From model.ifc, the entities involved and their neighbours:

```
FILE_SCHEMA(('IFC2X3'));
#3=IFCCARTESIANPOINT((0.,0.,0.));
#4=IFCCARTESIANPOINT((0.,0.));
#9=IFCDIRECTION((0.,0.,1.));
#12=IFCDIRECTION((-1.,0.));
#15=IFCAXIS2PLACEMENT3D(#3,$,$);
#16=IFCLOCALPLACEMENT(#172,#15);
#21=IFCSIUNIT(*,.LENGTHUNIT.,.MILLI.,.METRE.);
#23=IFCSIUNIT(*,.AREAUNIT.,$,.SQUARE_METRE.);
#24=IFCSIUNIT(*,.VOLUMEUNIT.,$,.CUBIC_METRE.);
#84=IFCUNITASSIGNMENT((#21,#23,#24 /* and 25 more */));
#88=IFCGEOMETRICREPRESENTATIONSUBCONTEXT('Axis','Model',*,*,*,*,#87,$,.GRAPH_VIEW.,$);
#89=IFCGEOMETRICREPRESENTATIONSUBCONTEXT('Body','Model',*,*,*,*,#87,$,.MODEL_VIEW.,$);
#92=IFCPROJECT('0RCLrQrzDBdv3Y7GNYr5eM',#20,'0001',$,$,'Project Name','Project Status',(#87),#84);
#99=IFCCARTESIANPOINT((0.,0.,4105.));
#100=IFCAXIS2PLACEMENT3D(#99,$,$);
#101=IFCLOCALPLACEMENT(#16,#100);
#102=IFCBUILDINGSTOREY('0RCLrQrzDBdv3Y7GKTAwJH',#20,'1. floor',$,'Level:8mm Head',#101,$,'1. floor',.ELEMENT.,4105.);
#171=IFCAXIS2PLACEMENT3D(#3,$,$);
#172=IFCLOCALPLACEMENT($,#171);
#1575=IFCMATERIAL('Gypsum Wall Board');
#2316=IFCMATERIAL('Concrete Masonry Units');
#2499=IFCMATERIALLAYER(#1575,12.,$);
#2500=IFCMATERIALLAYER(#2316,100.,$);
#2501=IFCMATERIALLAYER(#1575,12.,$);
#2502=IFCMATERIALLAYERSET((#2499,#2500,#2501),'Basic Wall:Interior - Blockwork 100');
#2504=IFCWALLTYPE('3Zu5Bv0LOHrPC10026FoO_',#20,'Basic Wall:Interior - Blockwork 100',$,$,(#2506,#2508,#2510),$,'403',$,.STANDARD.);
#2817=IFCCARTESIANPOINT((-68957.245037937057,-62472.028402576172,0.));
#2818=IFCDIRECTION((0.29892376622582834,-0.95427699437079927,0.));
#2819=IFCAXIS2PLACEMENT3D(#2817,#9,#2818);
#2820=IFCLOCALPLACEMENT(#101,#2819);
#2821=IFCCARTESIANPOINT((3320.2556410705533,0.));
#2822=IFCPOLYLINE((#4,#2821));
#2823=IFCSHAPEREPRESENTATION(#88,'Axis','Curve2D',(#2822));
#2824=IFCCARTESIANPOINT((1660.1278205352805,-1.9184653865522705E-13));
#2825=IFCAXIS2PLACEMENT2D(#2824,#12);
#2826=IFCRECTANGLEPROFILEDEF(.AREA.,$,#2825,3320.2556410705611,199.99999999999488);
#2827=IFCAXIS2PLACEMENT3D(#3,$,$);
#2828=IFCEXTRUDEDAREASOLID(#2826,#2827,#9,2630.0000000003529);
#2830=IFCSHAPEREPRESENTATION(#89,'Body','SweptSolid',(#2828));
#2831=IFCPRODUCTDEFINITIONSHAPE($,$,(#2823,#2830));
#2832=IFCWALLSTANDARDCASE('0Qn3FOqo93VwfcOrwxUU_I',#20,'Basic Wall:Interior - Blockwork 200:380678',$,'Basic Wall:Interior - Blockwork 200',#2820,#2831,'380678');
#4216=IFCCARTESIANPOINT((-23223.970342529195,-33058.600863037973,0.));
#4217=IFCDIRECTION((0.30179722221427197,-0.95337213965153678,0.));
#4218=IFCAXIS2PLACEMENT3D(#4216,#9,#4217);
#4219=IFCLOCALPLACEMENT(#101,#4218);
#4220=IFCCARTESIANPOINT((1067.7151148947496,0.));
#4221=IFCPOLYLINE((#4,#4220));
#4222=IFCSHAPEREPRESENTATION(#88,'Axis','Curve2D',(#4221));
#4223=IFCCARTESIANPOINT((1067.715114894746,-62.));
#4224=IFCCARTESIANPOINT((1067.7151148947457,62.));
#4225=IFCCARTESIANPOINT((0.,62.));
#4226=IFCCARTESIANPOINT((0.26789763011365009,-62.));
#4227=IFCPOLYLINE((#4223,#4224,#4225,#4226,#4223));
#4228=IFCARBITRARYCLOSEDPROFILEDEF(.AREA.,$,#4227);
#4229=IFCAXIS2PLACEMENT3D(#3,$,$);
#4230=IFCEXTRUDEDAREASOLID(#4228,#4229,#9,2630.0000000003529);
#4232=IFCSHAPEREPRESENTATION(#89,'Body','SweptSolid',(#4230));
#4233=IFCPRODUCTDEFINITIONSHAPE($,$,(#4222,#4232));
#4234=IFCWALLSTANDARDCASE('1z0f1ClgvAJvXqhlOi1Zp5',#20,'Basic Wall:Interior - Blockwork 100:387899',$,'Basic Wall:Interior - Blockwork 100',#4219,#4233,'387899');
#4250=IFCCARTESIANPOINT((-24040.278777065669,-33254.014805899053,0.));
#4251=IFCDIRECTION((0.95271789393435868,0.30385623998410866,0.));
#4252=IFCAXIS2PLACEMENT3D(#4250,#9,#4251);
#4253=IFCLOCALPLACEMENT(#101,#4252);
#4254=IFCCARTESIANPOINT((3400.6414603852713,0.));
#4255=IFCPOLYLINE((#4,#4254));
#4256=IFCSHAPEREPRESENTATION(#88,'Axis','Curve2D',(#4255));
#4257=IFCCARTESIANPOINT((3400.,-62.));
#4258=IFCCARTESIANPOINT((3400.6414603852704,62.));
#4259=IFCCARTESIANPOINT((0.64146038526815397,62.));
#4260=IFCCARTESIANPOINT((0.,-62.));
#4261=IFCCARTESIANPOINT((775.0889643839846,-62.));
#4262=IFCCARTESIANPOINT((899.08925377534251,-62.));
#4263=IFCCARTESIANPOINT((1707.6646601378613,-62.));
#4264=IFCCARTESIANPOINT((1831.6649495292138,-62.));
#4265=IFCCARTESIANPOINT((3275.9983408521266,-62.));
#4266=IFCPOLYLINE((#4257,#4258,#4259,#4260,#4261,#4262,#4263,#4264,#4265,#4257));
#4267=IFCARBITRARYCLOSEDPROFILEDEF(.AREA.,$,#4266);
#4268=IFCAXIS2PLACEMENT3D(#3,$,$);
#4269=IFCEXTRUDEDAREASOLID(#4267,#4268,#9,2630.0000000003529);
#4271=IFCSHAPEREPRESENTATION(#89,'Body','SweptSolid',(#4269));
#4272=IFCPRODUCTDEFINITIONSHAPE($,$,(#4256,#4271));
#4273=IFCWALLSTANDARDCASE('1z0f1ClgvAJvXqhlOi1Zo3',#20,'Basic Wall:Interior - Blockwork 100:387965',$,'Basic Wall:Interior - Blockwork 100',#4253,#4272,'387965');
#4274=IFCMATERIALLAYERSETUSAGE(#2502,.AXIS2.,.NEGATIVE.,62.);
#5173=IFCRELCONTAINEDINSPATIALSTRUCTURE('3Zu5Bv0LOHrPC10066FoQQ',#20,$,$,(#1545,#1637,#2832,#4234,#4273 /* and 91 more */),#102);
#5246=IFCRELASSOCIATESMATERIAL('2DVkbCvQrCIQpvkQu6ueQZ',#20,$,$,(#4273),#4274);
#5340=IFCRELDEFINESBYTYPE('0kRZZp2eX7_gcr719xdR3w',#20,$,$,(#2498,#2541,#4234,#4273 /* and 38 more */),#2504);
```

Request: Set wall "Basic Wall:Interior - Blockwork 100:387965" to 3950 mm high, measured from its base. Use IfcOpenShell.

```python
import ifcopenshell
import ifcopenshell.geom
import ifcopenshell.util.representation
import ifcopenshell.util.shape
import ifcopenshell.util.unit

model = ifcopenshell.open("model.ifc")
unit_scale = ifcopenshell.util.unit.calculate_unit_scale(model)
settings = ifcopenshell.geom.settings()


def volume(element):
    """Net volume in cubic metres, openings subtracted."""
    shape = ifcopenshell.geom.create_shape(settings, element)
    return ifcopenshell.util.shape.get_volume(shape.geometry)


wall = model.by_guid("1z0f1ClgvAJvXqhlOi1Zo3")
before = volume(wall)

body = ifcopenshell.util.representation.get_representation(wall, "Model", "Body")
solid = body.Items[0]
old_height = solid.Depth
solid.Depth = 3.95 / unit_scale
after = volume(wall)

print(f"height {old_height:g} -> {solid.Depth:g}, volume {before:.3f} -> {after:.3f} m3")

model.write("model_edited.ifc")
```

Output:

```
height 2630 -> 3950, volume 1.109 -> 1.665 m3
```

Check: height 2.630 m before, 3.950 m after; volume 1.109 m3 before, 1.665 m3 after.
